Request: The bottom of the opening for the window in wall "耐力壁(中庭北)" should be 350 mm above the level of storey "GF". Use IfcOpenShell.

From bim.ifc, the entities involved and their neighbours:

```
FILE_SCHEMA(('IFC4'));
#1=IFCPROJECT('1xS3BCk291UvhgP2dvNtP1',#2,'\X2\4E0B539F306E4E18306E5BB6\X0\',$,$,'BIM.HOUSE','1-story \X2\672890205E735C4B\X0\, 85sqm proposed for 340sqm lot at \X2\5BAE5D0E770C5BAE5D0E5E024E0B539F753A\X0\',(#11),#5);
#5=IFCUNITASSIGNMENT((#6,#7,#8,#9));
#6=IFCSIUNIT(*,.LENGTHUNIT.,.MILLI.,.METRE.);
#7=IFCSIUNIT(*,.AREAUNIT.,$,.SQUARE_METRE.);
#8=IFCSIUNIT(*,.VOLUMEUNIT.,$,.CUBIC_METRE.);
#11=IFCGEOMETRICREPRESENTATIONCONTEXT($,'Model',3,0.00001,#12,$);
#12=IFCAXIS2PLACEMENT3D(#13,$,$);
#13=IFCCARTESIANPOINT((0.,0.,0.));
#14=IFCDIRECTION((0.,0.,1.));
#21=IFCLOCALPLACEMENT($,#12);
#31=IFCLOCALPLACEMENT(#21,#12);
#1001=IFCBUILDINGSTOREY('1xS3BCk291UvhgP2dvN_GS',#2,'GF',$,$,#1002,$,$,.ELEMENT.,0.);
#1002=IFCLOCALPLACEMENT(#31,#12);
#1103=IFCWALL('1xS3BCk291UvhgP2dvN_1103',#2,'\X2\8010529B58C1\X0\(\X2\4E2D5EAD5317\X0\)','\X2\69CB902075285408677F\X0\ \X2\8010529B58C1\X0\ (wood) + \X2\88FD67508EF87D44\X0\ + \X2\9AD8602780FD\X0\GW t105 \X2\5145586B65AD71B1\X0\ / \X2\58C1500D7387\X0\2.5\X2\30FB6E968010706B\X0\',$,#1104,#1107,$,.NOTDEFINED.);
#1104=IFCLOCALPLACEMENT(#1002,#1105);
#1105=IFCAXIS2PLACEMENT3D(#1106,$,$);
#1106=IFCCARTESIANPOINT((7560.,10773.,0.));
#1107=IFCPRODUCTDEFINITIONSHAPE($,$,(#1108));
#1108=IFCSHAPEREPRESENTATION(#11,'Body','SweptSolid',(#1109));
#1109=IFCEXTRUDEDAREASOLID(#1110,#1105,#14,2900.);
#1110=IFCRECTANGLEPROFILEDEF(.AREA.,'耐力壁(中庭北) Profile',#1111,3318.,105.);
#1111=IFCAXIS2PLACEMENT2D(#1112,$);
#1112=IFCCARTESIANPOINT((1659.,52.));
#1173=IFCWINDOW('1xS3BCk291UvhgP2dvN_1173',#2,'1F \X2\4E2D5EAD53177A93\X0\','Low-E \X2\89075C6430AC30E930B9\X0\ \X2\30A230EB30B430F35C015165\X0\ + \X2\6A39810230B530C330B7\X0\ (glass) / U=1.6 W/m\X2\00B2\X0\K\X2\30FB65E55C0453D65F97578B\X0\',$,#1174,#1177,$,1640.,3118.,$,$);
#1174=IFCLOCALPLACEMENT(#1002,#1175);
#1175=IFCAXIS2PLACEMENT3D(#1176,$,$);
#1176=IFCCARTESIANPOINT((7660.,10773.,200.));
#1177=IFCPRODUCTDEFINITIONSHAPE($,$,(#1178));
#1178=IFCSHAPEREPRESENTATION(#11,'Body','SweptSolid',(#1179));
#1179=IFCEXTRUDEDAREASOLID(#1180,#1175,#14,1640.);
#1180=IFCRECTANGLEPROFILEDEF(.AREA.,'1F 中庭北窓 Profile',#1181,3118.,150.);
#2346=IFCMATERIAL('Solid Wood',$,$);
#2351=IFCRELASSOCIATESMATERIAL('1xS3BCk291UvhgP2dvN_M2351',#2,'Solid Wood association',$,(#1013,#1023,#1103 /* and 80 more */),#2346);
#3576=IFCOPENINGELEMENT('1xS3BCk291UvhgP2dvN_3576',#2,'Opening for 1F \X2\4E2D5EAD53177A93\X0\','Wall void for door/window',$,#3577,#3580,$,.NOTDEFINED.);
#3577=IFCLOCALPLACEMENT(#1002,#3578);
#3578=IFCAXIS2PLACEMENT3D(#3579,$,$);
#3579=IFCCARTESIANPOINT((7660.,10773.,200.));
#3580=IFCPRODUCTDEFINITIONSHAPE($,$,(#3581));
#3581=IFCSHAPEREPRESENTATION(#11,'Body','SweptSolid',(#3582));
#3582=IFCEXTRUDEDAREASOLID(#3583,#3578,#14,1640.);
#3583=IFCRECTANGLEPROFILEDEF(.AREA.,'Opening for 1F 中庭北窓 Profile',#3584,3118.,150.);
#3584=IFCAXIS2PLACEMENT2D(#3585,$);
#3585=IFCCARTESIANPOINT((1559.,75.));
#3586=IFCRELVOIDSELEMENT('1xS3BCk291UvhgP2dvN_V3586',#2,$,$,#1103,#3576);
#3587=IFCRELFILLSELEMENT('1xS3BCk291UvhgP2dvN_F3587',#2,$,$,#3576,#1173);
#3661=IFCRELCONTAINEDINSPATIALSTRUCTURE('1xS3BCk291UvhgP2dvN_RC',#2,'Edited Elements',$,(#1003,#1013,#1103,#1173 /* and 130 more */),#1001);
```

```python
import numpy as np
import ifcopenshell
import ifcopenshell.api.geometry
import ifcopenshell.geom
import ifcopenshell.util.element
import ifcopenshell.util.placement
import ifcopenshell.util.shape
import ifcopenshell.util.unit

model = ifcopenshell.open("bim.ifc")
unit_scale = ifcopenshell.util.unit.calculate_unit_scale(model)

window = model.by_id(1173)
opening = window.FillsVoids[0].RelatingOpeningElement
storey = ifcopenshell.util.element.get_container(window, ifc_class="IfcBuildingStorey")
level = ifcopenshell.util.placement.get_local_placement(storey.ObjectPlacement)[2, 3]

# The opening's origin need not be at the sill, so measure its lowest point.
shape = ifcopenshell.geom.create_shape(ifcopenshell.geom.settings(), opening)
bottom = ifcopenshell.util.shape.get_shape_bottom_elevation(shape, shape.geometry) / unit_scale
dz = level + 350.0 - bottom

shift = np.array([0.0, 0.0, dz])
# The window is not placed relative to its opening, so move both.
for product in (opening, window):
    matrix = ifcopenshell.util.placement.get_local_placement(product.ObjectPlacement)
    matrix[:3, 3] += shift
    ifcopenshell.api.geometry.edit_object_placement(model, product=product, matrix=matrix, is_si=False)

print(f"moved by {dz * unit_scale:+.3f} m")

model.write("bim_updated.ifc")
```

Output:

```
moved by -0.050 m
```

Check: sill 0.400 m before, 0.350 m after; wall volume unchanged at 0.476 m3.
